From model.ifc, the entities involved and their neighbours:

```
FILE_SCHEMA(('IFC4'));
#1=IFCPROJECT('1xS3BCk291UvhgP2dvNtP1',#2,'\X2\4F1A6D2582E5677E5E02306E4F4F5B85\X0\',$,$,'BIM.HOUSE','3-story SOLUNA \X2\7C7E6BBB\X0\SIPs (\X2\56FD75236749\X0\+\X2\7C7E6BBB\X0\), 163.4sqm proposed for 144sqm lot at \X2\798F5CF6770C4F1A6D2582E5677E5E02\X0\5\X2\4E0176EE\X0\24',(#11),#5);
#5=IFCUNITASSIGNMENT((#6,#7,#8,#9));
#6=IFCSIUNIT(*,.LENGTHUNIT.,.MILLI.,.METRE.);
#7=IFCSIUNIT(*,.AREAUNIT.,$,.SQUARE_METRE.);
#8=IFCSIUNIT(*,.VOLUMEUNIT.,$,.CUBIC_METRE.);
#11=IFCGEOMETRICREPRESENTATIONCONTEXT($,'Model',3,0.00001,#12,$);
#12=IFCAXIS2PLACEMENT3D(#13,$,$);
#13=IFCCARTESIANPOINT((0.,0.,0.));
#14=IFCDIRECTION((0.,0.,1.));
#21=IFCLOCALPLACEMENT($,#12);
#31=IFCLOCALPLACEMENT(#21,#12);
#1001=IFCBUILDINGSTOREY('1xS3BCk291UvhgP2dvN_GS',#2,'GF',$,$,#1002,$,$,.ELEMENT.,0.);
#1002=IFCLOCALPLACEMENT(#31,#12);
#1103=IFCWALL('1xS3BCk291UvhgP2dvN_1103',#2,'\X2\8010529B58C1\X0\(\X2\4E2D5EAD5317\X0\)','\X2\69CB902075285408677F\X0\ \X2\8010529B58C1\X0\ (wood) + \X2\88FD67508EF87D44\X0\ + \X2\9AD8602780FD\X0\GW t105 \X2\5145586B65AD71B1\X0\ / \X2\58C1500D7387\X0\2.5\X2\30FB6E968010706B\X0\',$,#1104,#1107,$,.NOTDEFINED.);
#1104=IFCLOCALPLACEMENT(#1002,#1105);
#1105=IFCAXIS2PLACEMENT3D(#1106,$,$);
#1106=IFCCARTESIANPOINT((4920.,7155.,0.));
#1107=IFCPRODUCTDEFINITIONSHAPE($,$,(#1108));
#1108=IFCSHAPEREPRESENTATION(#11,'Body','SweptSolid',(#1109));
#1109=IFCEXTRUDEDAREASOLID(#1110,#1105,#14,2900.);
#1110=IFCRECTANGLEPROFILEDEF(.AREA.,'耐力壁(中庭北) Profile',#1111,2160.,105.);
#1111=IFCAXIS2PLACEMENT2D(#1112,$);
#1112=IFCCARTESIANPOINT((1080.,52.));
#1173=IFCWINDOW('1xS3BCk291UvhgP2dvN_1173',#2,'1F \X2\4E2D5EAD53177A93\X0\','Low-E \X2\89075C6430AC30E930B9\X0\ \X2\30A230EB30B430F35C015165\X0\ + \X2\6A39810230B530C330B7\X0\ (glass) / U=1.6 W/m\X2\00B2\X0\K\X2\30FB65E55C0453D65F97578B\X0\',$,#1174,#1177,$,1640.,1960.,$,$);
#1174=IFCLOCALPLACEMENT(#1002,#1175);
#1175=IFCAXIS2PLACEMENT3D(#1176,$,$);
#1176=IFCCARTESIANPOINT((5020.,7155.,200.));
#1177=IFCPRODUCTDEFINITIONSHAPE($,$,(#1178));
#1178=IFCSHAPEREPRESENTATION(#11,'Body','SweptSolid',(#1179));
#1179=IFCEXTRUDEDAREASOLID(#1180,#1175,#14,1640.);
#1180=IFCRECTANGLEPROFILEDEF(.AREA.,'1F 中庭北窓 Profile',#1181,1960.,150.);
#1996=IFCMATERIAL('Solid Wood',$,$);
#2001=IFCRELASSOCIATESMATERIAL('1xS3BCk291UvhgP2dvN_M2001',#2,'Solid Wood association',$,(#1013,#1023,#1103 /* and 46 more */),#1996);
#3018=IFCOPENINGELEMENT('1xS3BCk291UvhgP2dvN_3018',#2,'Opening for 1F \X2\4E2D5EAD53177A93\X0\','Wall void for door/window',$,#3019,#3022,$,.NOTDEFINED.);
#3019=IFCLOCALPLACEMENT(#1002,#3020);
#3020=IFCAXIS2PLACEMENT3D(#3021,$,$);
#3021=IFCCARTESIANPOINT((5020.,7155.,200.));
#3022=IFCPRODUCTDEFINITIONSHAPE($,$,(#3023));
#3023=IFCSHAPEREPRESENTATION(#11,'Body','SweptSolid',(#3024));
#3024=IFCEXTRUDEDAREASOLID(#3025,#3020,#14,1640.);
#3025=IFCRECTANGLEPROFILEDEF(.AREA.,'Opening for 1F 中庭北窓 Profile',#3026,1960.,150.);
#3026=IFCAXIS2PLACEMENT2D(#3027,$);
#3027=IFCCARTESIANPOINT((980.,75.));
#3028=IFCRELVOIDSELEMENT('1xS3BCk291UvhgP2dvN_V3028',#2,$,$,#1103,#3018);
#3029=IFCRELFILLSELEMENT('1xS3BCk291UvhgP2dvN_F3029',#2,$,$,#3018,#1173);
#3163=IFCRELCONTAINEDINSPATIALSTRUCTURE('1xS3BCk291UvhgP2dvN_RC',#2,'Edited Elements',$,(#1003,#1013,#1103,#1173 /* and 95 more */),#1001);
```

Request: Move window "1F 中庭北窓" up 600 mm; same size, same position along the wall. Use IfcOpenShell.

```python
import numpy as np
import ifcopenshell
import ifcopenshell.api.geometry
import ifcopenshell.util.placement
import ifcopenshell.util.unit

model = ifcopenshell.open("model.ifc")
unit_scale = ifcopenshell.util.unit.calculate_unit_scale(model)

window = model.by_guid("1xS3BCk291UvhgP2dvN_1173")
opening = window.FillsVoids[0].RelatingOpeningElement
dz = 0.6 / unit_scale

shift = np.array([0.0, 0.0, dz])
# The window is not placed relative to its opening, so move both.
for product in (opening, window):
    matrix = ifcopenshell.util.placement.get_local_placement(product.ObjectPlacement)
    matrix[:3, 3] += shift
    ifcopenshell.api.geometry.edit_object_placement(model, product=product, matrix=matrix, is_si=False)

print(f"moved by {dz * unit_scale:+.3f} m")

model.write("model_rev.ifc")
```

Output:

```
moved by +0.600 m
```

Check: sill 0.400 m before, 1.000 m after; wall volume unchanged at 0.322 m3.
